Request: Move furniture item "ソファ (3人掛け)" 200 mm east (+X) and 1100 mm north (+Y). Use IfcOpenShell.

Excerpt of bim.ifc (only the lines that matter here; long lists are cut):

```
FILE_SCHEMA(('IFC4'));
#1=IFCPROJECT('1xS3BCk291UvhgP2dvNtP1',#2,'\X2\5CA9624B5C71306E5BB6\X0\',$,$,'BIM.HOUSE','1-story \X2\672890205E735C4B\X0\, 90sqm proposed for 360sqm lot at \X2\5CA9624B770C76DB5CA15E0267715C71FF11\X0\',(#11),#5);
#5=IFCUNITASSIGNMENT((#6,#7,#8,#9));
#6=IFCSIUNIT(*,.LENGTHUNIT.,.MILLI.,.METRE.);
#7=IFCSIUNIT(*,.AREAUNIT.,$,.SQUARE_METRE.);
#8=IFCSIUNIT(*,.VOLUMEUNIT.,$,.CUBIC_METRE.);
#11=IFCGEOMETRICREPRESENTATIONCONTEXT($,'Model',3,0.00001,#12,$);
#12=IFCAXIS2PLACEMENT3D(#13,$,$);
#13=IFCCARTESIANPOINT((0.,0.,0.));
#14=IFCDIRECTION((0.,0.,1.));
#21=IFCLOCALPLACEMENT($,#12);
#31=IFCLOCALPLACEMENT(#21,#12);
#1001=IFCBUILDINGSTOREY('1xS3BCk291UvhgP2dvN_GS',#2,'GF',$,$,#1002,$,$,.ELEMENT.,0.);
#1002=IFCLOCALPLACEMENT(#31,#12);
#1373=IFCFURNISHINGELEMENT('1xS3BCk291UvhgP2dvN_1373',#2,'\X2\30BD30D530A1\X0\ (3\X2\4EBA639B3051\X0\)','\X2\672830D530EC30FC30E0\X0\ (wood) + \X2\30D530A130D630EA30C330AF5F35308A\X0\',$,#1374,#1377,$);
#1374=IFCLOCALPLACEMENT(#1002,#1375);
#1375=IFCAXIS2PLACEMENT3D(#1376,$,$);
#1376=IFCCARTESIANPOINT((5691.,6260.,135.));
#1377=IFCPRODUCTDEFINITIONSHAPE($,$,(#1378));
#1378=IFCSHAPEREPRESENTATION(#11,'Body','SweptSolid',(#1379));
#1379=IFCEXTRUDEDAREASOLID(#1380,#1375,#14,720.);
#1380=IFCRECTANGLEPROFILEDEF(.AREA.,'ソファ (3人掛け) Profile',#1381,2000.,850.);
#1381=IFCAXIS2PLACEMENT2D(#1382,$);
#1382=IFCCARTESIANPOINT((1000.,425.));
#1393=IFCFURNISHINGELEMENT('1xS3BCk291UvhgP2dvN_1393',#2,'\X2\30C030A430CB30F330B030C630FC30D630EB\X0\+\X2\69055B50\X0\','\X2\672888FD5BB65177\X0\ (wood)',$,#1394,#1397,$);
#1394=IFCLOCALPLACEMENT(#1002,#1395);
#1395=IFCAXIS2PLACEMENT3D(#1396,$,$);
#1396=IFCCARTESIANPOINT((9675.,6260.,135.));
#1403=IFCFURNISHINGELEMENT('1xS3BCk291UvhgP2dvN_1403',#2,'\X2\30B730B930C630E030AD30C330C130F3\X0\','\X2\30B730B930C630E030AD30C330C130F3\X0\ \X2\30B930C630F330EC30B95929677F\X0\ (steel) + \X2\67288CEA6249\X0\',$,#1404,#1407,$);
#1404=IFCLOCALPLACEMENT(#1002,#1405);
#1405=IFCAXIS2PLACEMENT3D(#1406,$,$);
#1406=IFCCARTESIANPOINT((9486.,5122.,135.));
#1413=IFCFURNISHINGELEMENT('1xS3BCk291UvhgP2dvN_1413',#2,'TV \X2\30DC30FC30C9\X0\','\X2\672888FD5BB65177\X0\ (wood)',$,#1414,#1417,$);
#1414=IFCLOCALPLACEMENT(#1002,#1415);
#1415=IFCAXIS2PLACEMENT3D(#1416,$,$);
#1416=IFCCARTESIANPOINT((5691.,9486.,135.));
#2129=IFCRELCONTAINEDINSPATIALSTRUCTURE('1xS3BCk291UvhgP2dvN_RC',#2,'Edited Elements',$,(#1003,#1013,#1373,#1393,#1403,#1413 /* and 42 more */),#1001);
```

```python
import ifcopenshell
import ifcopenshell.api.geometry
import ifcopenshell.util.placement
import ifcopenshell.util.unit

model = ifcopenshell.open("bim.ifc")
unit_scale = ifcopenshell.util.unit.calculate_unit_scale(model)

item = model.by_id(1373)
matrix = ifcopenshell.util.placement.get_local_placement(item.ObjectPlacement)
matrix[0, 3] += 0.2 / unit_scale
matrix[1, 3] += 1.1 / unit_scale
ifcopenshell.api.geometry.edit_object_placement(model, product=item, matrix=matrix, is_si=False)

print(ifcopenshell.util.placement.get_local_placement(item.ObjectPlacement).round(3) + 0.0)

model.write("bim_v2.ifc")
```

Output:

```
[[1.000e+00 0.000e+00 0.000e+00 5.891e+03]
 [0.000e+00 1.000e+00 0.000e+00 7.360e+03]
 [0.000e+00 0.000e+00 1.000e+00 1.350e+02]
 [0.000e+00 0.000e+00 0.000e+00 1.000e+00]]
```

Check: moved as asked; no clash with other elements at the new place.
